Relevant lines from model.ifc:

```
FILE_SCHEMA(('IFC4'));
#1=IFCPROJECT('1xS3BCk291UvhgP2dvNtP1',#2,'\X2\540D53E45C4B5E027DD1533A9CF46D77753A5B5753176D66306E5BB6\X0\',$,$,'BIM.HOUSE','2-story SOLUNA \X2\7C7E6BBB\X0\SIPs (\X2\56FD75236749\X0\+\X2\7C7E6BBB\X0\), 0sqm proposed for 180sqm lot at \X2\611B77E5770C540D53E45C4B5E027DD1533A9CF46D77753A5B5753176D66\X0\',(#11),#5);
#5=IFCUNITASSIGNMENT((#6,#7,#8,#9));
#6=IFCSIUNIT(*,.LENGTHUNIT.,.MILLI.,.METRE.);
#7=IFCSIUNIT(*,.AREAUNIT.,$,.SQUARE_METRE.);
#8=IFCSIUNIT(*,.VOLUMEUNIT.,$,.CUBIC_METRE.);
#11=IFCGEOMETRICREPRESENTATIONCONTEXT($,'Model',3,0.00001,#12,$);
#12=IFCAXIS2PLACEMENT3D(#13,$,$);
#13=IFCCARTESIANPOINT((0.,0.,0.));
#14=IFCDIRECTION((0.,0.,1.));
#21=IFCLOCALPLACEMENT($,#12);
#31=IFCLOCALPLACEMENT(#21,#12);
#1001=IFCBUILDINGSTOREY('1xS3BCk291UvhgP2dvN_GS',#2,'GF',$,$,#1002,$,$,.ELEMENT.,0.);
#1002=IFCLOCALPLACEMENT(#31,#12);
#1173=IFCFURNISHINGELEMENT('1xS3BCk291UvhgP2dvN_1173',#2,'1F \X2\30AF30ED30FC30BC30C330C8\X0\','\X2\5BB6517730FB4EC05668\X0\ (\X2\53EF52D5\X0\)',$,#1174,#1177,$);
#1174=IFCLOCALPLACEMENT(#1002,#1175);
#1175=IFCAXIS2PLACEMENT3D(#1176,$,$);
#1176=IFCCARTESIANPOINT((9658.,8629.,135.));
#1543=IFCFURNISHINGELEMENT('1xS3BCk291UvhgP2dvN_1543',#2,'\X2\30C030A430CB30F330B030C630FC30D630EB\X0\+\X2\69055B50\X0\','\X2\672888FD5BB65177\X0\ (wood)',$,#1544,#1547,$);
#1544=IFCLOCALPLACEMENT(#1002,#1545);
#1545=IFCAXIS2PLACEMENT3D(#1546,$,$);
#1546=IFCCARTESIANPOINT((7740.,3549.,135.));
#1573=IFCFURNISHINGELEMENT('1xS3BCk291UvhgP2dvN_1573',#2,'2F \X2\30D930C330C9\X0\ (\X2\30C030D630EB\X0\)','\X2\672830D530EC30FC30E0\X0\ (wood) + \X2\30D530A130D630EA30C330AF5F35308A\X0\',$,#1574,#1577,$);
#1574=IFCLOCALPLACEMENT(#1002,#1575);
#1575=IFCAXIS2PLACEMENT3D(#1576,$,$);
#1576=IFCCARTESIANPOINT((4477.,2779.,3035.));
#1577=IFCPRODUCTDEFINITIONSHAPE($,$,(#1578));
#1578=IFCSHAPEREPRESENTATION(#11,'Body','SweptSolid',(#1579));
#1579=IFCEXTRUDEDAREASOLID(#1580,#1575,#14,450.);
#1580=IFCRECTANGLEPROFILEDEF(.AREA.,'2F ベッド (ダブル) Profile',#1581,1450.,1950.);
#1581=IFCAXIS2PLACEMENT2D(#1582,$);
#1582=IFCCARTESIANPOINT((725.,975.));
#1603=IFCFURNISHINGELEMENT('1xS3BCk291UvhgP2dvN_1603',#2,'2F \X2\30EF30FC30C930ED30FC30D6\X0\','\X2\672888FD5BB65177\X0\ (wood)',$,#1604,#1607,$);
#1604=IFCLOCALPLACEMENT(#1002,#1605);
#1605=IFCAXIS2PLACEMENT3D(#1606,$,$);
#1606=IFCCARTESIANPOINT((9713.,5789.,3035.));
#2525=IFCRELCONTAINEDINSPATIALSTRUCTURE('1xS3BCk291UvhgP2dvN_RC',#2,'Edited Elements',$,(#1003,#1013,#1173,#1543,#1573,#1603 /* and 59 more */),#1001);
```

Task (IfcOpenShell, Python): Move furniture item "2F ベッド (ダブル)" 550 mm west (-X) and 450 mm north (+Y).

```python
import ifcopenshell
import ifcopenshell.api.geometry
import ifcopenshell.util.placement

model = ifcopenshell.open("model.ifc")

item = model.by_guid("1xS3BCk291UvhgP2dvN_1573")
matrix = ifcopenshell.util.placement.get_local_placement(item.ObjectPlacement)
matrix[0, 3] -= 550.0
matrix[1, 3] += 450.0
ifcopenshell.api.geometry.edit_object_placement(model, product=item, matrix=matrix, is_si=False)

print(ifcopenshell.util.placement.get_local_placement(item.ObjectPlacement).round(3) + 0.0)

model.write("model_v2.ifc")
```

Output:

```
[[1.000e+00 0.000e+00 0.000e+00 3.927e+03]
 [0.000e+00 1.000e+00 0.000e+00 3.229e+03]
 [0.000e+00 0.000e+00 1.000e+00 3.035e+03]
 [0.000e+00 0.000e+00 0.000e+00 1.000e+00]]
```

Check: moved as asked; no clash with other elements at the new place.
